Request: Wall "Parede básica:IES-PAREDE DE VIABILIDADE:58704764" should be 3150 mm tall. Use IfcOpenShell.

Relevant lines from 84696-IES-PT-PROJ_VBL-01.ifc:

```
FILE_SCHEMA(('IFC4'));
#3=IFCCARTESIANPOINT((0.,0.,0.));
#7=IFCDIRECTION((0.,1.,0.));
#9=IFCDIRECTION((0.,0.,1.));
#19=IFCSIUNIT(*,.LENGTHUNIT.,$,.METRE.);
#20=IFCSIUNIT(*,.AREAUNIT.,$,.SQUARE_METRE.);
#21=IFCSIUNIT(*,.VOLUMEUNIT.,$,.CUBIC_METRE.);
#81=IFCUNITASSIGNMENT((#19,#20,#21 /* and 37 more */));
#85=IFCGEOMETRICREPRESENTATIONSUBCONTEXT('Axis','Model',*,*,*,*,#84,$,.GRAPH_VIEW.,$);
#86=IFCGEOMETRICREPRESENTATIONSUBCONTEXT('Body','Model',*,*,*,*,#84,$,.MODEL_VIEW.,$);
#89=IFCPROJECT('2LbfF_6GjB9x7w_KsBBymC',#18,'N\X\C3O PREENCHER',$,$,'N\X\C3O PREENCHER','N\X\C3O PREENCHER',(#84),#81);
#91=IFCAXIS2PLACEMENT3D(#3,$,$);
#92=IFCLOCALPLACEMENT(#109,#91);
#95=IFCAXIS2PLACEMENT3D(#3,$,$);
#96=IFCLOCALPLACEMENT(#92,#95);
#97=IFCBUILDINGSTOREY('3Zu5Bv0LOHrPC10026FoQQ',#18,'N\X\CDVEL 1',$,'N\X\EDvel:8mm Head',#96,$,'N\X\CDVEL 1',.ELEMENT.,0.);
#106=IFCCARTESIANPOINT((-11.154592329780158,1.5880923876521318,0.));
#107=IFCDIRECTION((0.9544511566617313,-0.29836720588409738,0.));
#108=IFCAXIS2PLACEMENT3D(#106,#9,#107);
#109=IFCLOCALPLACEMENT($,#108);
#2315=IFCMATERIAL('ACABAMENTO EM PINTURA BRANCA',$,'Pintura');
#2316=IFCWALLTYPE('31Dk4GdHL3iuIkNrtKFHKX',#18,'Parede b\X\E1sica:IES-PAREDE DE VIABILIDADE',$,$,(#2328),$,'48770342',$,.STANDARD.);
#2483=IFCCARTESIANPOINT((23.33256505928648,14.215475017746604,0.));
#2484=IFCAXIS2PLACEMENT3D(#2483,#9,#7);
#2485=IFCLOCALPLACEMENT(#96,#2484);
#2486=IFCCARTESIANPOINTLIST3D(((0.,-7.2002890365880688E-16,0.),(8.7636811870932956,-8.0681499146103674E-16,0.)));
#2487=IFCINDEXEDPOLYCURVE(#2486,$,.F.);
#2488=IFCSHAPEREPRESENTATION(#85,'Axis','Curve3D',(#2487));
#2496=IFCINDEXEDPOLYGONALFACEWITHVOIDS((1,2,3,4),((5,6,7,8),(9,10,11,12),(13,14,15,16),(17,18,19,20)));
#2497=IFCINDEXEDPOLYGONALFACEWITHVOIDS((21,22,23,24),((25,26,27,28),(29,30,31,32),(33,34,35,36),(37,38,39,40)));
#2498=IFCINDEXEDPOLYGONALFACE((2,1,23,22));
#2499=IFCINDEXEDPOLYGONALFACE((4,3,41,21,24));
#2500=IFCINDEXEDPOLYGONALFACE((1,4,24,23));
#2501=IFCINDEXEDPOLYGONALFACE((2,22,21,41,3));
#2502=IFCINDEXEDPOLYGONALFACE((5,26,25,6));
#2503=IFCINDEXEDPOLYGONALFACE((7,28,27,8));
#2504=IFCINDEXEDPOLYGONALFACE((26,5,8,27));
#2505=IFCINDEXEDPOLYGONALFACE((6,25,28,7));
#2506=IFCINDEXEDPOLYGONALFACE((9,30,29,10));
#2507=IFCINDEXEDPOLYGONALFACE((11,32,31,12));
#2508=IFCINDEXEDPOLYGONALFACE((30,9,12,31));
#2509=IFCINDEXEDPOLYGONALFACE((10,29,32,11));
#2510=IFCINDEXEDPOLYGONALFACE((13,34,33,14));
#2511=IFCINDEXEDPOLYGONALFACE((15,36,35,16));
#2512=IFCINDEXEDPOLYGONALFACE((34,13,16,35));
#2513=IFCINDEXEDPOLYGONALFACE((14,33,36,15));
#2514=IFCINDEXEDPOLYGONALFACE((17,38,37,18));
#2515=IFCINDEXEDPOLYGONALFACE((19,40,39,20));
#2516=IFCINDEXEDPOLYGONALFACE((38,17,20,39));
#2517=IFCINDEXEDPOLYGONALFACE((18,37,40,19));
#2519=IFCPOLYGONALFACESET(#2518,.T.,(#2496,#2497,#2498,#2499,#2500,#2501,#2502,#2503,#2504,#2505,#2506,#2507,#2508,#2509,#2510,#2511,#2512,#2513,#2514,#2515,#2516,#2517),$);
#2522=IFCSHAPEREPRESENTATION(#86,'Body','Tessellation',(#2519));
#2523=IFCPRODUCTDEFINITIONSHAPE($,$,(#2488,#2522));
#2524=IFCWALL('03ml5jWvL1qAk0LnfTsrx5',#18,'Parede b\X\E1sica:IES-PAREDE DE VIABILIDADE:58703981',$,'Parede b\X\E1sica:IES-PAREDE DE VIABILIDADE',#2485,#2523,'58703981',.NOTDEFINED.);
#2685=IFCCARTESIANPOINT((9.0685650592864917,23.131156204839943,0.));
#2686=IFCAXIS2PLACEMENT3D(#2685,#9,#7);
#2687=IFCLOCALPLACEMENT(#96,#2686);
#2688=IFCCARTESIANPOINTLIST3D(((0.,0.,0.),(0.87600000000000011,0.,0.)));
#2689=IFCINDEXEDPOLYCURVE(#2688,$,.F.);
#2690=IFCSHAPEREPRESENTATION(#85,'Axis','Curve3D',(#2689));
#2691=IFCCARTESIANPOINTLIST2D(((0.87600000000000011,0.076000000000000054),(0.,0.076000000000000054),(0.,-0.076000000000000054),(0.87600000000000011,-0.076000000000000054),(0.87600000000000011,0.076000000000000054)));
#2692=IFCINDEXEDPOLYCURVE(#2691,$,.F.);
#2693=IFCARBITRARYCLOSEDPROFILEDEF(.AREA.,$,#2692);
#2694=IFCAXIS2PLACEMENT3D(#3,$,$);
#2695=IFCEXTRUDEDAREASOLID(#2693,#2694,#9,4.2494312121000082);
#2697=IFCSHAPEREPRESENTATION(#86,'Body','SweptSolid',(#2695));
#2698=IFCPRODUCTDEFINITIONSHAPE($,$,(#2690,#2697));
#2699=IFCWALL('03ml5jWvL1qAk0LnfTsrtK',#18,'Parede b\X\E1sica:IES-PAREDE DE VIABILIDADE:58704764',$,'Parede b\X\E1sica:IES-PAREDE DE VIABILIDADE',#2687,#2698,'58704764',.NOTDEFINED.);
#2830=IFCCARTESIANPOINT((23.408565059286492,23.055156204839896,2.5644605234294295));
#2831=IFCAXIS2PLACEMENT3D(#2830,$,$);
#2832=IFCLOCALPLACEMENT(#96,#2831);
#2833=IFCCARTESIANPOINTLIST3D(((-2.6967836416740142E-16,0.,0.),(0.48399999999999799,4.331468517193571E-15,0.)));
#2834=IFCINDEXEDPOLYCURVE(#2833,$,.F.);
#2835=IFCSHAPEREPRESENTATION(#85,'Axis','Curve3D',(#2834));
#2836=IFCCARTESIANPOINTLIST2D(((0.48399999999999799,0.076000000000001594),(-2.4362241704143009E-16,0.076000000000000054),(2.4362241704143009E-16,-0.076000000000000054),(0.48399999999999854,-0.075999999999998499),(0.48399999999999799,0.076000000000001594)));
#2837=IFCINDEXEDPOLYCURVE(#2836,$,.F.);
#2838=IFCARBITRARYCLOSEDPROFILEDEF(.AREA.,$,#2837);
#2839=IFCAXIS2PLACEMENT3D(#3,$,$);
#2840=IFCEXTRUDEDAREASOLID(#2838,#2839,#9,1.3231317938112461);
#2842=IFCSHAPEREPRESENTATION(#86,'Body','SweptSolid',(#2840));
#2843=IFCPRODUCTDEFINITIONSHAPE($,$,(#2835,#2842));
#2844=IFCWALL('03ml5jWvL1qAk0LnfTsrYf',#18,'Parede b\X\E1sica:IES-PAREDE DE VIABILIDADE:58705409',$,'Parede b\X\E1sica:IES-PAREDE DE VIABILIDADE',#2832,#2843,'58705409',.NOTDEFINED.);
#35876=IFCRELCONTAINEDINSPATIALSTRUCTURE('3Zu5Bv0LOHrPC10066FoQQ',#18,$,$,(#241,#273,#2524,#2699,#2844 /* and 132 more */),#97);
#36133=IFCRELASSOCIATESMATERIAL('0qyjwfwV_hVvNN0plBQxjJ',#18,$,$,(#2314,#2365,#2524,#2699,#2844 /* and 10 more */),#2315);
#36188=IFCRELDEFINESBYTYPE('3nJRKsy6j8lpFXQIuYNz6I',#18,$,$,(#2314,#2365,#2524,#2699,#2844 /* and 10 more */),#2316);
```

```python
import ifcopenshell
import ifcopenshell.geom
import ifcopenshell.util.representation
import ifcopenshell.util.shape
import ifcopenshell.util.unit

model = ifcopenshell.open("84696-IES-PT-PROJ_VBL-01.ifc")
unit_scale = ifcopenshell.util.unit.calculate_unit_scale(model)
settings = ifcopenshell.geom.settings()


def volume(element):
    """Net volume in cubic metres, openings subtracted."""
    shape = ifcopenshell.geom.create_shape(settings, element)
    return ifcopenshell.util.shape.get_volume(shape.geometry)


wall = model.by_id(2699)
before = volume(wall)

body = ifcopenshell.util.representation.get_representation(wall, "Model", "Body")
solid = body.Items[0]
old_height = solid.Depth
solid.Depth = 3.15 / unit_scale
after = volume(wall)

print(f"height {old_height:g} -> {solid.Depth:g}, volume {before:.3f} -> {after:.3f} m3")

model.write("84696-IES-PT-PROJ_VBL-01_v2.ifc")
```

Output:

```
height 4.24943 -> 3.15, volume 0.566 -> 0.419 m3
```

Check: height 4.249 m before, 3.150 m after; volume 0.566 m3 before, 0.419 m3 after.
